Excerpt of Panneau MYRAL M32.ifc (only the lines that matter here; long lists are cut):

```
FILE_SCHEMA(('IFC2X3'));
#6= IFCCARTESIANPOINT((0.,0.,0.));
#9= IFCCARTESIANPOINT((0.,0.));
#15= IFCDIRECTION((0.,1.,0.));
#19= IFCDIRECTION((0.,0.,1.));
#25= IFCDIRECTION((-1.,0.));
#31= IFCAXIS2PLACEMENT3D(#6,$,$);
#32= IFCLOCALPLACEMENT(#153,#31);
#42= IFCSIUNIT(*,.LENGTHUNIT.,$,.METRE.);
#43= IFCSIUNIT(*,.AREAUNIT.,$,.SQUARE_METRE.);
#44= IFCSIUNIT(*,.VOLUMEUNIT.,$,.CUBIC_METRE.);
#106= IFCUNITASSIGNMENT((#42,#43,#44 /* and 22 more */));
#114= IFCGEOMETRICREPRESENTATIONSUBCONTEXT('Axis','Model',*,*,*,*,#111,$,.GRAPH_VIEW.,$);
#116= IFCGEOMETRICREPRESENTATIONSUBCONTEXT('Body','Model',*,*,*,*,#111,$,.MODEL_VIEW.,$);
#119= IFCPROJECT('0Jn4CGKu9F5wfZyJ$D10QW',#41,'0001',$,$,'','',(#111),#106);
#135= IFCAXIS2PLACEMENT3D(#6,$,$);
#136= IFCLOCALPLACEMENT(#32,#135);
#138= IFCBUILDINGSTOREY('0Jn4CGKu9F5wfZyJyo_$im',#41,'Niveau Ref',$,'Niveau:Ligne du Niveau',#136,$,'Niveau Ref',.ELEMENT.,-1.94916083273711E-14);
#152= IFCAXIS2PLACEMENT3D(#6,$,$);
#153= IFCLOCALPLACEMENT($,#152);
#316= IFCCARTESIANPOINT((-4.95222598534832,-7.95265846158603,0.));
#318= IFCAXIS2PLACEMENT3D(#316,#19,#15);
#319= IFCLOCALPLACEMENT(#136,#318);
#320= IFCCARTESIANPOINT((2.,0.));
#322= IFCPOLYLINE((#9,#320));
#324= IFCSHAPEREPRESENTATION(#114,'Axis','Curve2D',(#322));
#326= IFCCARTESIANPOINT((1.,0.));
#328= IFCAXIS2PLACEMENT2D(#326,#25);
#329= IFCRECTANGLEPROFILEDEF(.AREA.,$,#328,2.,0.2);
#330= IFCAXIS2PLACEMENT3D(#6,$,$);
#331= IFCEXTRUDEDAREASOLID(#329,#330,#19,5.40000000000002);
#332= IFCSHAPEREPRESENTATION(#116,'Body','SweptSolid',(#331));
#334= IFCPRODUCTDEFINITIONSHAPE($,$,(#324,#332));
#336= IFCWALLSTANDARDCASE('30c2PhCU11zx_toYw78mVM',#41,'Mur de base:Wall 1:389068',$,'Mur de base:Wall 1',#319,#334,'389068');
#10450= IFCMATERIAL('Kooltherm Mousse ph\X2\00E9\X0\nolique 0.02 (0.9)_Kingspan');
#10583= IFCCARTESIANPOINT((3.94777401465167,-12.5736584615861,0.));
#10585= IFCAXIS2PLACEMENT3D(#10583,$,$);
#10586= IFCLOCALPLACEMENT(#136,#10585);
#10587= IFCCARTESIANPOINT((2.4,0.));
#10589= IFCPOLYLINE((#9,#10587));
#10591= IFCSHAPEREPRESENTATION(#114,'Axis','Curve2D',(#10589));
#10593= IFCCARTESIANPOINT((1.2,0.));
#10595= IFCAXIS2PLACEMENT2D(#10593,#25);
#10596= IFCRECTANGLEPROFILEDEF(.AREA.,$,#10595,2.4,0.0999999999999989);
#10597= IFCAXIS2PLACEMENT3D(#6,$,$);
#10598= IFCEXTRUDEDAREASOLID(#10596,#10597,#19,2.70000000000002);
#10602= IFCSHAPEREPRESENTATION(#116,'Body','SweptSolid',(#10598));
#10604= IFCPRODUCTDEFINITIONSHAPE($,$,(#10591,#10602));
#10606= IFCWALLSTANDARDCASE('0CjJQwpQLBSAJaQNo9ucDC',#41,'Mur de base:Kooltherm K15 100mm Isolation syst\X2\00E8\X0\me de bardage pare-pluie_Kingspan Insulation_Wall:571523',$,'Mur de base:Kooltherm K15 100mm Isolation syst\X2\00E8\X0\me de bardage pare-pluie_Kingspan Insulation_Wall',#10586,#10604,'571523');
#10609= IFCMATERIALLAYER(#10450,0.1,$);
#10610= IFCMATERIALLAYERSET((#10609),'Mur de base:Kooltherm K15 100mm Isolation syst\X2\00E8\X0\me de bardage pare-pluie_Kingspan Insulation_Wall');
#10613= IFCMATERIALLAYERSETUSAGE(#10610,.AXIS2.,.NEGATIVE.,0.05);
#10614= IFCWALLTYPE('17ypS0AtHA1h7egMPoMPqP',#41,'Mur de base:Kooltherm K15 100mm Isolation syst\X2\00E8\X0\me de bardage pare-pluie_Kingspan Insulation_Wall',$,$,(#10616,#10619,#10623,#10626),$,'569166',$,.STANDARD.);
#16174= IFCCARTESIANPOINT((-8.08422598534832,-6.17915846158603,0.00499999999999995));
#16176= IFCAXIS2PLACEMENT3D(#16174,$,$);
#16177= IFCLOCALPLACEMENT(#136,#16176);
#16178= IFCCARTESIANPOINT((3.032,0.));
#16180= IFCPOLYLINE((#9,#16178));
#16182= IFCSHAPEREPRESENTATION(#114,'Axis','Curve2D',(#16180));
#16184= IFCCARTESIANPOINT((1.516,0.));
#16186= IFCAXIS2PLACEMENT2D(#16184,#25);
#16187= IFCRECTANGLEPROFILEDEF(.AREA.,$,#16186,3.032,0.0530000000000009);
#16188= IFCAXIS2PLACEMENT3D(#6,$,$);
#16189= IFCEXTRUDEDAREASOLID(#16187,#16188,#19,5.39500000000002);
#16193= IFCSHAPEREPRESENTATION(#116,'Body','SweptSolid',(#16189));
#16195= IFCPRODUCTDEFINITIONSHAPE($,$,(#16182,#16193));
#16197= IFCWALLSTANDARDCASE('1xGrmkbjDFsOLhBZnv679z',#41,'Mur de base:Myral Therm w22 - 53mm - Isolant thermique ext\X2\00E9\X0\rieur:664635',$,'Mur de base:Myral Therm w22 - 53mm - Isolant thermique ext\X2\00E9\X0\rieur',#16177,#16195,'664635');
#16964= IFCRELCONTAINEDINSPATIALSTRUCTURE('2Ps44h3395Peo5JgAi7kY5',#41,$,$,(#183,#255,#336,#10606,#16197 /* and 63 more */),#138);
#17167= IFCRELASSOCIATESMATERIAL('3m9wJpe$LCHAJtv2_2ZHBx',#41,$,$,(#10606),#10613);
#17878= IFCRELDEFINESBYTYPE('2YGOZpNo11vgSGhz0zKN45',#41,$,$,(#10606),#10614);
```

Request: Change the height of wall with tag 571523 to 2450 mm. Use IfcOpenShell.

```python
import ifcopenshell
import ifcopenshell.geom
import ifcopenshell.util.representation
import ifcopenshell.util.shape
import ifcopenshell.util.unit

model = ifcopenshell.open("Panneau MYRAL M32.ifc")
unit_scale = ifcopenshell.util.unit.calculate_unit_scale(model)
settings = ifcopenshell.geom.settings()


def volume(element):
    """Net volume in cubic metres, openings subtracted."""
    shape = ifcopenshell.geom.create_shape(settings, element)
    return ifcopenshell.util.shape.get_volume(shape.geometry)


wall = model.by_guid("0CjJQwpQLBSAJaQNo9ucDC")
before = volume(wall)

body = ifcopenshell.util.representation.get_representation(wall, "Model", "Body")
solid = body.Items[0]
old_height = solid.Depth
solid.Depth = 2.45 / unit_scale
after = volume(wall)

print(f"height {old_height:g} -> {solid.Depth:g}, volume {before:.3f} -> {after:.3f} m3")

model.write("Panneau MYRAL M32_rev.ifc")
```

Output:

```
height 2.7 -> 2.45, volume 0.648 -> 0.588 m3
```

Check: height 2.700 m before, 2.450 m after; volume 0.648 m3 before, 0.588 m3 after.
